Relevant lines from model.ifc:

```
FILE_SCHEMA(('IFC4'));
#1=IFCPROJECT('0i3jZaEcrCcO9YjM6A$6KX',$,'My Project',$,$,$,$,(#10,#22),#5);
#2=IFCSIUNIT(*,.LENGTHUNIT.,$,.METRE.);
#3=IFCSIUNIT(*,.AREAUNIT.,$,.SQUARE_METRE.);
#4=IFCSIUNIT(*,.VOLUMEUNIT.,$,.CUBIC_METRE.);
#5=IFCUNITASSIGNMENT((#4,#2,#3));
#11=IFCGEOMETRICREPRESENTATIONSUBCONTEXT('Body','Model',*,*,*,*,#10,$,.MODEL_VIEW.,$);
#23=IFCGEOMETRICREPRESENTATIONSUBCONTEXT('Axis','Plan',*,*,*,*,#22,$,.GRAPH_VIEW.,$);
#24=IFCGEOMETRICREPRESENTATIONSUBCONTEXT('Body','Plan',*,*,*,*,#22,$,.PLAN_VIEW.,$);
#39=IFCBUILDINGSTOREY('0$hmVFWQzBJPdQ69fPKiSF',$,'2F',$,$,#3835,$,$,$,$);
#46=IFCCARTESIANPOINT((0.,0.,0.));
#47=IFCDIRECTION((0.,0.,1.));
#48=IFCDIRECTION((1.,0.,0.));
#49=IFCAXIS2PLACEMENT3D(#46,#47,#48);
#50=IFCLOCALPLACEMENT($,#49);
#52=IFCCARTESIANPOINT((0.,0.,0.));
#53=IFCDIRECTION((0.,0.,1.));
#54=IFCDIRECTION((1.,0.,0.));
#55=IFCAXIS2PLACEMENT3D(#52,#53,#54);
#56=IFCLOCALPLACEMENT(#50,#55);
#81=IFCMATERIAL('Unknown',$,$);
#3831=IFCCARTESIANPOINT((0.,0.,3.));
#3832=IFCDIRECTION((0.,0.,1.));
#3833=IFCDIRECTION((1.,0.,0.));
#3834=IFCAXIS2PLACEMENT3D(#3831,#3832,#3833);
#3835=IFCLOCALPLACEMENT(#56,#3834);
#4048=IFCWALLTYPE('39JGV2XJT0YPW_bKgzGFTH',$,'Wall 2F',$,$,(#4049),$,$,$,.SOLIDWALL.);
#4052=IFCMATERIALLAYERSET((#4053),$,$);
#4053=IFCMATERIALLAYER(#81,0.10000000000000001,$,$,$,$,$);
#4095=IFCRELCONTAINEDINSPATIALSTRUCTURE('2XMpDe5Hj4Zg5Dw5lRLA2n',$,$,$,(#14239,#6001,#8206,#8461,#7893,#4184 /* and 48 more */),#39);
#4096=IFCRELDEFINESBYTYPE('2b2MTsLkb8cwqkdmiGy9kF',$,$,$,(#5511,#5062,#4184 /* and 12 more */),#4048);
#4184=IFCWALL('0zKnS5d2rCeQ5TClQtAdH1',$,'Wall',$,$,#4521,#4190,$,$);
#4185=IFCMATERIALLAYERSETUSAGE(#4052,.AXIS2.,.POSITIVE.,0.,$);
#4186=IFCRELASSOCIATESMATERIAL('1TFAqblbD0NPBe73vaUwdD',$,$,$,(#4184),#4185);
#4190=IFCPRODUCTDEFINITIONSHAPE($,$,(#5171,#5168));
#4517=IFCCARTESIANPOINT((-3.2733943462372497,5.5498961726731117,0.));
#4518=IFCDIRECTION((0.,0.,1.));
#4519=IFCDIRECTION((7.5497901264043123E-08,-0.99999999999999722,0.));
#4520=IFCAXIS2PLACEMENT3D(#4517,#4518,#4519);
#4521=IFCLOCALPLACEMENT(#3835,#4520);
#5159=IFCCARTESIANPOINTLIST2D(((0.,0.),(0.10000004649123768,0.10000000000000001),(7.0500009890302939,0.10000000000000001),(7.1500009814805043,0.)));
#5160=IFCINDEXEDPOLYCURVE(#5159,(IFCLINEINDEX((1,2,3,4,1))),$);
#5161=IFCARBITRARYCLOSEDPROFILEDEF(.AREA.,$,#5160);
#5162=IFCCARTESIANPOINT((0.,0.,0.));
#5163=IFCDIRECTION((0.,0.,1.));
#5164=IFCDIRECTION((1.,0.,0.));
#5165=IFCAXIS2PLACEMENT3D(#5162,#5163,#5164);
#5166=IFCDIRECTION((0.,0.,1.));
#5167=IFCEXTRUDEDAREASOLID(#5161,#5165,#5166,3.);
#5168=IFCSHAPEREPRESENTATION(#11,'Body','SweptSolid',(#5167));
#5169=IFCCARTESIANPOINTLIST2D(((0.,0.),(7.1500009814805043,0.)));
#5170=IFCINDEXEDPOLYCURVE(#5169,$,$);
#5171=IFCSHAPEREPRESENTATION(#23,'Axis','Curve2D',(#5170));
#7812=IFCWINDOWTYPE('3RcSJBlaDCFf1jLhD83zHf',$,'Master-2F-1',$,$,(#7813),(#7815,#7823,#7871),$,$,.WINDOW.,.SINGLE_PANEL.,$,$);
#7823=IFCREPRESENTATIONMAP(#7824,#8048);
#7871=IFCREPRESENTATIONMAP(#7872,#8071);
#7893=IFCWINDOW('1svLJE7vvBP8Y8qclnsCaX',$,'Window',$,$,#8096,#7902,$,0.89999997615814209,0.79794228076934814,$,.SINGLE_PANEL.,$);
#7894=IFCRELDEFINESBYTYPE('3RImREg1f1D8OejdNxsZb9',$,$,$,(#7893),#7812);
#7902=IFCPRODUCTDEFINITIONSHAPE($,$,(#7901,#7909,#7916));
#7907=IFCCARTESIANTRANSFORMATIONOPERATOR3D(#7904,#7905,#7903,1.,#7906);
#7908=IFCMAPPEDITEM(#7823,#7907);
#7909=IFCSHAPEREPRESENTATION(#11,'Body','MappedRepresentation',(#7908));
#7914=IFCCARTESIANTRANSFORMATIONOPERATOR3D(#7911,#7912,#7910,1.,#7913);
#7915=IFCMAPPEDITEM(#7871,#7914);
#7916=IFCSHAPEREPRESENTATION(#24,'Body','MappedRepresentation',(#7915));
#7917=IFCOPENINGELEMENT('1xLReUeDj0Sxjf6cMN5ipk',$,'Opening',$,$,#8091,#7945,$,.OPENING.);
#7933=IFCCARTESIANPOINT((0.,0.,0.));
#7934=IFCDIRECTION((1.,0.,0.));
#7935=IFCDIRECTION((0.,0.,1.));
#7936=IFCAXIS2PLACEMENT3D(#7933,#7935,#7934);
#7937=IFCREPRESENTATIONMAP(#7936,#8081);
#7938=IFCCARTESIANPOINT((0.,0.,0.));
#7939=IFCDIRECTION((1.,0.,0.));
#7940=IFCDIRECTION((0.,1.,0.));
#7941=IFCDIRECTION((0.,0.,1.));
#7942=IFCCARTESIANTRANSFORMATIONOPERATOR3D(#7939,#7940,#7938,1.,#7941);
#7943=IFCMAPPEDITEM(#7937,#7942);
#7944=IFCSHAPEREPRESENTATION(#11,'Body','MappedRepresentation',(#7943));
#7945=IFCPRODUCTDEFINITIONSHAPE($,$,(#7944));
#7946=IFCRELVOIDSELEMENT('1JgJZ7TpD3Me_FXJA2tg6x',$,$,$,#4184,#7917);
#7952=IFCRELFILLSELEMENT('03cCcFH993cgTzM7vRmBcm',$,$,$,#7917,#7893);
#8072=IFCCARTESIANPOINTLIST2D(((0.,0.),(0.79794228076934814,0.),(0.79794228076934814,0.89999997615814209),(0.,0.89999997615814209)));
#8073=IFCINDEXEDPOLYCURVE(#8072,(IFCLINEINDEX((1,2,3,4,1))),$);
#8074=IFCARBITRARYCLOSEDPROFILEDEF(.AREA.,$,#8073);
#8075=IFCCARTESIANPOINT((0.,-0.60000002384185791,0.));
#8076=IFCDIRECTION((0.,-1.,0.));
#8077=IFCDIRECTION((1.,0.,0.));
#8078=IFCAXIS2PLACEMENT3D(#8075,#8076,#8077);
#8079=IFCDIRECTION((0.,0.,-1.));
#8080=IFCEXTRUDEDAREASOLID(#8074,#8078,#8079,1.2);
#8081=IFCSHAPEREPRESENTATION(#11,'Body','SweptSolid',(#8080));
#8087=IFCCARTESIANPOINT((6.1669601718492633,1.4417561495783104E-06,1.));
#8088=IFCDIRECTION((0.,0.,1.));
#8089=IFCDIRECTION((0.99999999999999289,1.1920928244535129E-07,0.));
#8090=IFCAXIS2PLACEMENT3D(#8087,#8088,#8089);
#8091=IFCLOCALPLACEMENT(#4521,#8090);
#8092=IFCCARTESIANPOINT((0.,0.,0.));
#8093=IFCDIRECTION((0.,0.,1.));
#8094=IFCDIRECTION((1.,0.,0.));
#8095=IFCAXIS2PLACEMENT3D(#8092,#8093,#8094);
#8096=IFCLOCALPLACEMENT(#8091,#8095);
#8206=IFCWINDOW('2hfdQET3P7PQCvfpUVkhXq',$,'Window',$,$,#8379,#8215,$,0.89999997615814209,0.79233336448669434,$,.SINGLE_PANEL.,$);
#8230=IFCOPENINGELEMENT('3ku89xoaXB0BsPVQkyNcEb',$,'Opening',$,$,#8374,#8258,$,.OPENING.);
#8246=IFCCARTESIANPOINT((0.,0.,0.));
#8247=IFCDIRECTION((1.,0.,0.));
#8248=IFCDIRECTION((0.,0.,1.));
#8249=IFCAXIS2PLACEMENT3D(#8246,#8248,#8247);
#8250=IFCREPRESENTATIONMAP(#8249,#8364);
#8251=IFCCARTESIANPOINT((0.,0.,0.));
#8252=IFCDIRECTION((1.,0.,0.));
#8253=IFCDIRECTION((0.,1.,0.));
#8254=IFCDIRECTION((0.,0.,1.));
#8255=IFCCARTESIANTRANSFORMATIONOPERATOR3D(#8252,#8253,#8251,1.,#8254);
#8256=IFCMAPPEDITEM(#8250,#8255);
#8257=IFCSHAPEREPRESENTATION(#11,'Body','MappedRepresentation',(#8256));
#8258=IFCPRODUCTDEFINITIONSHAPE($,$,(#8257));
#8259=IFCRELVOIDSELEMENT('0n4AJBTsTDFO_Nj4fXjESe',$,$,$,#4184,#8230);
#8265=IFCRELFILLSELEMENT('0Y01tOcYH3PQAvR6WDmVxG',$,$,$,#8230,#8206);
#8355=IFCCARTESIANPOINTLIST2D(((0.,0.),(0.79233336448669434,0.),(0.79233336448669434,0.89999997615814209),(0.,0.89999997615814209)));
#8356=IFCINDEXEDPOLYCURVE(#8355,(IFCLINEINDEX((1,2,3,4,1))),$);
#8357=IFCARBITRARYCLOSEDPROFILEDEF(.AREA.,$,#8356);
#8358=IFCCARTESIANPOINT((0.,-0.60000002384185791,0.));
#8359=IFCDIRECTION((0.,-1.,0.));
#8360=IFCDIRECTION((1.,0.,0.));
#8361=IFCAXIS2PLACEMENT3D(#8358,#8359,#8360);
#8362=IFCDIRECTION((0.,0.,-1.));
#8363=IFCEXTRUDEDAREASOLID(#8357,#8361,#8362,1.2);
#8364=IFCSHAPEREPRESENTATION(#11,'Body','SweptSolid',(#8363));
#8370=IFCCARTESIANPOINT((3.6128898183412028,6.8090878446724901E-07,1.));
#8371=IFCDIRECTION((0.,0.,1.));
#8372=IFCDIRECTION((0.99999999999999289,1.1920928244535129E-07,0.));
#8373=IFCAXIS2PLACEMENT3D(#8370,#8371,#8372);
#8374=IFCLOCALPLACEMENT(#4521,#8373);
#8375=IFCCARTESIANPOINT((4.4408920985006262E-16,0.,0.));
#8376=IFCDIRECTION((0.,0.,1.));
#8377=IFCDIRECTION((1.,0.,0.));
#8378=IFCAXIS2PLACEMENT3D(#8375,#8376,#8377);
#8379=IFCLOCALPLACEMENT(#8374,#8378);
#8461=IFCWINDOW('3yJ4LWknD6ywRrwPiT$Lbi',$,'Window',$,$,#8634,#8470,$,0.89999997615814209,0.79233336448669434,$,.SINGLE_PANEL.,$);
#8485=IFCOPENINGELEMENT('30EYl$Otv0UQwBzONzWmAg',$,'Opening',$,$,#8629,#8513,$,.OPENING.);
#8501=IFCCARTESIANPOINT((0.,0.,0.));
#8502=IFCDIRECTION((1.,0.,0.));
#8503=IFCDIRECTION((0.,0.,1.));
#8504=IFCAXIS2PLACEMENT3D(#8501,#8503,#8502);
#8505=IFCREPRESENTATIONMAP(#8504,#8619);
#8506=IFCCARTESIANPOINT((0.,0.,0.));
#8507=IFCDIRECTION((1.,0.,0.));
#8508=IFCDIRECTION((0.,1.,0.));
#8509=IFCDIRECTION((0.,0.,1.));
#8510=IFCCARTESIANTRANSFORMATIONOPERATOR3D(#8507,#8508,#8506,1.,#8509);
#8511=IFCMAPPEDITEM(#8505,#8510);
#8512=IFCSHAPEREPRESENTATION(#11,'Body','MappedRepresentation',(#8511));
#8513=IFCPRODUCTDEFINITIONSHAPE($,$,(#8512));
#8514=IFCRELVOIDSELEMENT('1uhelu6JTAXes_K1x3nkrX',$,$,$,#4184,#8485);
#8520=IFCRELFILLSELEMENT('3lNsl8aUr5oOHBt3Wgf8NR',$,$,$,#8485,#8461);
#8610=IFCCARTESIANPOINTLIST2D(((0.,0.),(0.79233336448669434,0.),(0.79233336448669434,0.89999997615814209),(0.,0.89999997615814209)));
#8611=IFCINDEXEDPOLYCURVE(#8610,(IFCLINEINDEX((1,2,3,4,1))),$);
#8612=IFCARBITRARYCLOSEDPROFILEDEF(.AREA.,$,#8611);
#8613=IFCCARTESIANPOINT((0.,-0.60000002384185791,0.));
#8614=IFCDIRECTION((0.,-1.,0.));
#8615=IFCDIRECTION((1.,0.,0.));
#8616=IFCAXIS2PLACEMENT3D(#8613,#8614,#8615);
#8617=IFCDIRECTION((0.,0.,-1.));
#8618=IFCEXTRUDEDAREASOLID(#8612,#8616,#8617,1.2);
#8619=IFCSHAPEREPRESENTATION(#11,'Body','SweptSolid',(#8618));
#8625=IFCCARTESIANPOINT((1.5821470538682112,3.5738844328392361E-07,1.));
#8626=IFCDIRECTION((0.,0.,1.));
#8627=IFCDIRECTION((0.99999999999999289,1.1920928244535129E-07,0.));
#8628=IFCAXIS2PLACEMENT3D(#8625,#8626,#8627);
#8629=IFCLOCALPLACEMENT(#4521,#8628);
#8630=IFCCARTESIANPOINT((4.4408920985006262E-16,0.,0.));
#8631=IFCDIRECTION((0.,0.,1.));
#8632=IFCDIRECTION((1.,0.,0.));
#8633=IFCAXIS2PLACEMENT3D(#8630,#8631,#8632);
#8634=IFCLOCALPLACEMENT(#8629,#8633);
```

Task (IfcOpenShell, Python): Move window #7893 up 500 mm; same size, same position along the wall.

```python
import numpy as np
import ifcopenshell
import ifcopenshell.api.geometry
import ifcopenshell.util.placement
import ifcopenshell.util.unit

model = ifcopenshell.open("model.ifc")
unit_scale = ifcopenshell.util.unit.calculate_unit_scale(model)

window = model.by_guid("1svLJE7vvBP8Y8qclnsCaX")
opening = window.FillsVoids[0].RelatingOpeningElement
dz = 0.5

shift = np.array([0.0, 0.0, dz])
# The window is placed relative to its opening, so it follows when the opening moves.
matrix = ifcopenshell.util.placement.get_local_placement(opening.ObjectPlacement)
matrix[:3, 3] += shift
ifcopenshell.api.geometry.edit_object_placement(
    model, product=opening, matrix=matrix, is_si=False, should_transform_children=True
)

print(f"moved by {dz * unit_scale:+.3f} m")

model.write("model-out.ifc")
```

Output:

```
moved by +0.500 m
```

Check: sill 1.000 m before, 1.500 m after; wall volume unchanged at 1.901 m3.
